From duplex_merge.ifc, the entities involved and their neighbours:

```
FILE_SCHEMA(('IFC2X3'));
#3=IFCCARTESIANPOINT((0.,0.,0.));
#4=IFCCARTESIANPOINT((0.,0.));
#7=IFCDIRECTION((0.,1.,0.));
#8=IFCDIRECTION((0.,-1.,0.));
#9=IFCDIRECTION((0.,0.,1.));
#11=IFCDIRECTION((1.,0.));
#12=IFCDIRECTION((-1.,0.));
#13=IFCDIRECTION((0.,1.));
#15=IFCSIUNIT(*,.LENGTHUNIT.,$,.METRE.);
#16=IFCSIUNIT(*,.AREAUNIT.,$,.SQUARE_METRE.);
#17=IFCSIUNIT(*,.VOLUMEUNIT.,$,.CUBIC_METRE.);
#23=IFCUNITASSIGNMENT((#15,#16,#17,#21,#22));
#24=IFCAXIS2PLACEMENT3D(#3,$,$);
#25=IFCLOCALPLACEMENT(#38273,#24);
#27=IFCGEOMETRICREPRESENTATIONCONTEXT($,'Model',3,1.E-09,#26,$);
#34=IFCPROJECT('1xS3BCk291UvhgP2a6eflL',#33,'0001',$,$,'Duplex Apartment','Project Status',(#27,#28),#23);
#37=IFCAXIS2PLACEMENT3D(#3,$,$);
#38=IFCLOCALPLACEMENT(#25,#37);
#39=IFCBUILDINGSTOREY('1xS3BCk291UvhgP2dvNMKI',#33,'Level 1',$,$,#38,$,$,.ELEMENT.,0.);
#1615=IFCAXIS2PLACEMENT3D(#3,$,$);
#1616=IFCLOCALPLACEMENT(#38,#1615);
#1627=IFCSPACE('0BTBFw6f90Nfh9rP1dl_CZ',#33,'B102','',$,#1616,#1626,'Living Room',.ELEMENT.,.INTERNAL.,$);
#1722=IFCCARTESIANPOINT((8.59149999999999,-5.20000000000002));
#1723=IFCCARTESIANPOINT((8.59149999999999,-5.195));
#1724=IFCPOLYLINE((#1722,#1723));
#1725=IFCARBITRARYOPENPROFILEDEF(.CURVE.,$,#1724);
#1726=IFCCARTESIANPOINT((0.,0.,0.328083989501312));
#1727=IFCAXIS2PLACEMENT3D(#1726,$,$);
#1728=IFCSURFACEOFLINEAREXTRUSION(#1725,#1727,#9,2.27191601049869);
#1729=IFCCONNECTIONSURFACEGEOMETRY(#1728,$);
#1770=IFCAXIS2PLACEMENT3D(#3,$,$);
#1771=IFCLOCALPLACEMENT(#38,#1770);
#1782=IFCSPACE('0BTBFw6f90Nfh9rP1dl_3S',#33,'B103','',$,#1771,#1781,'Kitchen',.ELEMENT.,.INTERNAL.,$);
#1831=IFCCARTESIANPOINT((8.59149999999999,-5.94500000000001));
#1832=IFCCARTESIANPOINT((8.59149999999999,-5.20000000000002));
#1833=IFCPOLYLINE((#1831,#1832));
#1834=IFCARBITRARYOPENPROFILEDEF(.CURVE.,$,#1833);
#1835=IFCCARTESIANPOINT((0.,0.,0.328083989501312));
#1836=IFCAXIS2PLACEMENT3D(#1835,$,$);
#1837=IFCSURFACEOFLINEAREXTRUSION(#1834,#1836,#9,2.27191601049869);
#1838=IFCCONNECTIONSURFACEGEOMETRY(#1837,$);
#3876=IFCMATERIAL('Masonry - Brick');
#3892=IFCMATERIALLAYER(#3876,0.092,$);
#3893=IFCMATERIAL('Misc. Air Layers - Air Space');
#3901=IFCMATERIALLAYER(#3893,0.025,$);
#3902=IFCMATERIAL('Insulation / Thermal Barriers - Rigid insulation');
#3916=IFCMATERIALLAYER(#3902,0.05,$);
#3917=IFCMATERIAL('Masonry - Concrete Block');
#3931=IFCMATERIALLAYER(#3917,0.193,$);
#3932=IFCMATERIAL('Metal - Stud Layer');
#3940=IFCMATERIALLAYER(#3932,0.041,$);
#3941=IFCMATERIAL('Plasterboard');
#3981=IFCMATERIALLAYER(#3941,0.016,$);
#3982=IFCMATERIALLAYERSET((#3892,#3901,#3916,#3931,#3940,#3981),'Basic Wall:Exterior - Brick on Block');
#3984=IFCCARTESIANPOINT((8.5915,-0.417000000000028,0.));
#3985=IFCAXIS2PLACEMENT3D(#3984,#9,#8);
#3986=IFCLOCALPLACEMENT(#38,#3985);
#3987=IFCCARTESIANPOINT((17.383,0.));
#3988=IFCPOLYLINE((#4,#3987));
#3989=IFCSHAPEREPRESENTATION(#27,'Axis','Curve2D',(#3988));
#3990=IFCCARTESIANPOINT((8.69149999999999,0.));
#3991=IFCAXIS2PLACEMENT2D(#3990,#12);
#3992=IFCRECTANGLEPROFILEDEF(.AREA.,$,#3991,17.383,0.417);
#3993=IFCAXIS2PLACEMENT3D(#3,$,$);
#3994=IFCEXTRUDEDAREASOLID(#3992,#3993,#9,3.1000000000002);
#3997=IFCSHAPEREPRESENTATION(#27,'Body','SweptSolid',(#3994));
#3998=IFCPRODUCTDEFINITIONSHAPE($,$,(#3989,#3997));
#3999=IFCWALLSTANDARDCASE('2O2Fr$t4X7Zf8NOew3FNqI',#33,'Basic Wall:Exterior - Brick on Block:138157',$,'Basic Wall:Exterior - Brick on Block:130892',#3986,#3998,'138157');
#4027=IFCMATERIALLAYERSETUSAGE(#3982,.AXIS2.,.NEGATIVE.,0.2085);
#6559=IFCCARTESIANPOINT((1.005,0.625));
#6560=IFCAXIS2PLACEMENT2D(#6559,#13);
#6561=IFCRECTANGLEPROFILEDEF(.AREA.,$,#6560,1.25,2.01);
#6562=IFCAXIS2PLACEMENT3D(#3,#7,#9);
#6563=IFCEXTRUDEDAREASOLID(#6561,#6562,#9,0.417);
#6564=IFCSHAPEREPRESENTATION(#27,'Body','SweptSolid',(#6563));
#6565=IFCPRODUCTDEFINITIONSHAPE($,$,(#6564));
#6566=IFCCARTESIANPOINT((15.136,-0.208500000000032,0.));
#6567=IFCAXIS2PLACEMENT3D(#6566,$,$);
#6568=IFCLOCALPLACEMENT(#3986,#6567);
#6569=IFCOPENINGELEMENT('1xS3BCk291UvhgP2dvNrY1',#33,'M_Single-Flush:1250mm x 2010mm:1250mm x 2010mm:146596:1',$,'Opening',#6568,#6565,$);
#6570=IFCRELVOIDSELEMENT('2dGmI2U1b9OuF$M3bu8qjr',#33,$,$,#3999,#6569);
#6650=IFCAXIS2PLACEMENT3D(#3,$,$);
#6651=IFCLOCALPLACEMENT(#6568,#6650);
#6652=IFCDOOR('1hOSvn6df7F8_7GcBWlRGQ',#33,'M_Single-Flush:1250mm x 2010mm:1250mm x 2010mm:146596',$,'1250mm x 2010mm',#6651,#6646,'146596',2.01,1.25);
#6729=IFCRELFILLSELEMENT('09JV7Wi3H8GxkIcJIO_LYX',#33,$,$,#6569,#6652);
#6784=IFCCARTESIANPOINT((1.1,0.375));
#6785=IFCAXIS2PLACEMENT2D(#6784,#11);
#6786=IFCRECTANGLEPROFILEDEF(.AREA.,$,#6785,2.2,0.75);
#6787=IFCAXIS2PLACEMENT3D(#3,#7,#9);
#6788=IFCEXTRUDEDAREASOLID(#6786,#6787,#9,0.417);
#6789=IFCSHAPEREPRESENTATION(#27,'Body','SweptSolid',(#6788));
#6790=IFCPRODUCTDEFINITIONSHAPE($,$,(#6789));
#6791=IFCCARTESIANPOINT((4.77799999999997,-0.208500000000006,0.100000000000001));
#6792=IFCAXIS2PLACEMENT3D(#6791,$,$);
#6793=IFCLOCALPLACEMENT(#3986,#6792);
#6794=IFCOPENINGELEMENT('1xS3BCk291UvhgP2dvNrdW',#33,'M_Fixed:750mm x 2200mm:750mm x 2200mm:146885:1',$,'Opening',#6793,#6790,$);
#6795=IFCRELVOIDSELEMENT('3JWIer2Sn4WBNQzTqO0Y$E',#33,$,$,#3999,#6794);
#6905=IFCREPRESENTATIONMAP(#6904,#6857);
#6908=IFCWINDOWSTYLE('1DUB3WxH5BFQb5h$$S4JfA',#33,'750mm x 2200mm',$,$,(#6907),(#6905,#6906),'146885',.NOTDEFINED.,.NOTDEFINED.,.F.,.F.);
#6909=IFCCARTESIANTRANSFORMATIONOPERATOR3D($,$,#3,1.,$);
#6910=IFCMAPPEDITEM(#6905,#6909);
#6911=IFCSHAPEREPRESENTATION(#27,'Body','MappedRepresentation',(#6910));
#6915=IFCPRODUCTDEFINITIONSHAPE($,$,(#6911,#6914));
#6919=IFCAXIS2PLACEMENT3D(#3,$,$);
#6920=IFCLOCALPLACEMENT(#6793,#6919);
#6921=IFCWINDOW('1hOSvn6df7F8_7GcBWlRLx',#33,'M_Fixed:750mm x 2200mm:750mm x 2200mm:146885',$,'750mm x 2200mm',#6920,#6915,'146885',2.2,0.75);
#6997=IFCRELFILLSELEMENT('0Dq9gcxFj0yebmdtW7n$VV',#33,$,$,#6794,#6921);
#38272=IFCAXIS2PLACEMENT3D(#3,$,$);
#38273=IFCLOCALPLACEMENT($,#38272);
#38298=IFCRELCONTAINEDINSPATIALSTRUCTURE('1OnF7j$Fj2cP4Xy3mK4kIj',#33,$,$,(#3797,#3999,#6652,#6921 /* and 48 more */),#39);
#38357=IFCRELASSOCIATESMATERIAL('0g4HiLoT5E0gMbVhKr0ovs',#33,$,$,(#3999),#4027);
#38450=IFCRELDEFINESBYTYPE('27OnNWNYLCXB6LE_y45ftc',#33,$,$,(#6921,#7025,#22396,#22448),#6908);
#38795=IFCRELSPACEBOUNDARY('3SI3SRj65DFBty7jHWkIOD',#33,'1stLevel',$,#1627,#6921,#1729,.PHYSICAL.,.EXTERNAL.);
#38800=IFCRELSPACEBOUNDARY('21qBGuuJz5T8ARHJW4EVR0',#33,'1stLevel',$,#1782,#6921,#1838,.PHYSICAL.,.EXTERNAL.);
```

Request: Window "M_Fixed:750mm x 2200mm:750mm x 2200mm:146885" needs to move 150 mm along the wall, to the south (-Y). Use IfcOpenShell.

```python
import numpy as np
import ifcopenshell
import ifcopenshell.api.geometry
import ifcopenshell.util.placement

model = ifcopenshell.open("duplex_merge.ifc")

window = model.by_guid("1hOSvn6df7F8_7GcBWlRLx")
opening = window.FillsVoids[0].RelatingOpeningElement
wall = opening.VoidsElements[0].RelatingBuildingElement

wall_matrix = ifcopenshell.util.placement.get_local_placement(wall.ObjectPlacement)
shift = wall_matrix[:3, 0] * 0.15
before = ifcopenshell.util.placement.get_local_placement(window.ObjectPlacement)[:3, 3].copy()

# The window is placed relative to its opening, so it follows when the opening moves.
matrix = ifcopenshell.util.placement.get_local_placement(opening.ObjectPlacement)
matrix[:3, 3] += shift
ifcopenshell.api.geometry.edit_object_placement(
    model, product=opening, matrix=matrix, is_si=False, should_transform_children=True
)

# Space boundary surfaces are stored in each space's coordinates; move them too.
for rel in window.ProvidesBoundaries:
    if not rel.ConnectionGeometry:
        continue
    surface = rel.ConnectionGeometry.SurfaceOnRelatingElement
    space_matrix = ifcopenshell.util.placement.get_local_placement(rel.RelatingSpace.ObjectPlacement)
    point = np.array(surface.Position.Location.Coordinates) + space_matrix[:3, :3].T @ shift
    surface.Position = model.createIfcAxis2Placement3D(
        model.createIfcCartesianPoint(point.tolist()), surface.Position.Axis, surface.Position.RefDirection
    )

after = ifcopenshell.util.placement.get_local_placement(window.ObjectPlacement)[:3, 3]
print("window moved by", (after - before).round(3) + 0.0)

model.write("duplex_merge-out.ifc")
```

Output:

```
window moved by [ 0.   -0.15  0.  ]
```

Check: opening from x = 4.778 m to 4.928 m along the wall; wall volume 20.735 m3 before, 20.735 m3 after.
